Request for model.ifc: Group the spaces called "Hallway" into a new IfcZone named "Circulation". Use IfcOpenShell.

First a look at what the model holds.

```python
import ifcopenshell

model = ifcopenshell.open("model.ifc")
print(model.schema)
seen = {}
for space in model.by_type("IfcSpace"):
    seen[space.LongName] = seen.get(space.LongName, 0) + 1
for name, count in sorted(seen.items(), key=str):
    print(count, "x", name)
print("zones:", [z.Name for z in model.by_type("IfcZone")][:20])
```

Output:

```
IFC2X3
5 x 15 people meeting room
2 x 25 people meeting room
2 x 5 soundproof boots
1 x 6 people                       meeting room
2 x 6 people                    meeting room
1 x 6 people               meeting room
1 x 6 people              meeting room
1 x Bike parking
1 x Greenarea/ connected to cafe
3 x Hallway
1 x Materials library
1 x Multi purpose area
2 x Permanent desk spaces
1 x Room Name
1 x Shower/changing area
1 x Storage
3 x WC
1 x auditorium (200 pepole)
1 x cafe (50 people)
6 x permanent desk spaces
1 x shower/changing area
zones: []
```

```python
import ifcopenshell
import ifcopenshell.api.group
import ifcopenshell.api.root

model = ifcopenshell.open("model.ifc")

names = {"Hallway"}
spaces = [s for s in model.by_type("IfcSpace") if s.LongName in names]

zone = ifcopenshell.api.root.create_entity(model, ifc_class="IfcZone", name="Circulation")
ifcopenshell.api.group.assign_group(model, products=spaces, group=zone)
print(len(spaces), "spaces in", zone.Name)

model.write("model-out.ifc")
```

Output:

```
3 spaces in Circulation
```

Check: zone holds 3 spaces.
